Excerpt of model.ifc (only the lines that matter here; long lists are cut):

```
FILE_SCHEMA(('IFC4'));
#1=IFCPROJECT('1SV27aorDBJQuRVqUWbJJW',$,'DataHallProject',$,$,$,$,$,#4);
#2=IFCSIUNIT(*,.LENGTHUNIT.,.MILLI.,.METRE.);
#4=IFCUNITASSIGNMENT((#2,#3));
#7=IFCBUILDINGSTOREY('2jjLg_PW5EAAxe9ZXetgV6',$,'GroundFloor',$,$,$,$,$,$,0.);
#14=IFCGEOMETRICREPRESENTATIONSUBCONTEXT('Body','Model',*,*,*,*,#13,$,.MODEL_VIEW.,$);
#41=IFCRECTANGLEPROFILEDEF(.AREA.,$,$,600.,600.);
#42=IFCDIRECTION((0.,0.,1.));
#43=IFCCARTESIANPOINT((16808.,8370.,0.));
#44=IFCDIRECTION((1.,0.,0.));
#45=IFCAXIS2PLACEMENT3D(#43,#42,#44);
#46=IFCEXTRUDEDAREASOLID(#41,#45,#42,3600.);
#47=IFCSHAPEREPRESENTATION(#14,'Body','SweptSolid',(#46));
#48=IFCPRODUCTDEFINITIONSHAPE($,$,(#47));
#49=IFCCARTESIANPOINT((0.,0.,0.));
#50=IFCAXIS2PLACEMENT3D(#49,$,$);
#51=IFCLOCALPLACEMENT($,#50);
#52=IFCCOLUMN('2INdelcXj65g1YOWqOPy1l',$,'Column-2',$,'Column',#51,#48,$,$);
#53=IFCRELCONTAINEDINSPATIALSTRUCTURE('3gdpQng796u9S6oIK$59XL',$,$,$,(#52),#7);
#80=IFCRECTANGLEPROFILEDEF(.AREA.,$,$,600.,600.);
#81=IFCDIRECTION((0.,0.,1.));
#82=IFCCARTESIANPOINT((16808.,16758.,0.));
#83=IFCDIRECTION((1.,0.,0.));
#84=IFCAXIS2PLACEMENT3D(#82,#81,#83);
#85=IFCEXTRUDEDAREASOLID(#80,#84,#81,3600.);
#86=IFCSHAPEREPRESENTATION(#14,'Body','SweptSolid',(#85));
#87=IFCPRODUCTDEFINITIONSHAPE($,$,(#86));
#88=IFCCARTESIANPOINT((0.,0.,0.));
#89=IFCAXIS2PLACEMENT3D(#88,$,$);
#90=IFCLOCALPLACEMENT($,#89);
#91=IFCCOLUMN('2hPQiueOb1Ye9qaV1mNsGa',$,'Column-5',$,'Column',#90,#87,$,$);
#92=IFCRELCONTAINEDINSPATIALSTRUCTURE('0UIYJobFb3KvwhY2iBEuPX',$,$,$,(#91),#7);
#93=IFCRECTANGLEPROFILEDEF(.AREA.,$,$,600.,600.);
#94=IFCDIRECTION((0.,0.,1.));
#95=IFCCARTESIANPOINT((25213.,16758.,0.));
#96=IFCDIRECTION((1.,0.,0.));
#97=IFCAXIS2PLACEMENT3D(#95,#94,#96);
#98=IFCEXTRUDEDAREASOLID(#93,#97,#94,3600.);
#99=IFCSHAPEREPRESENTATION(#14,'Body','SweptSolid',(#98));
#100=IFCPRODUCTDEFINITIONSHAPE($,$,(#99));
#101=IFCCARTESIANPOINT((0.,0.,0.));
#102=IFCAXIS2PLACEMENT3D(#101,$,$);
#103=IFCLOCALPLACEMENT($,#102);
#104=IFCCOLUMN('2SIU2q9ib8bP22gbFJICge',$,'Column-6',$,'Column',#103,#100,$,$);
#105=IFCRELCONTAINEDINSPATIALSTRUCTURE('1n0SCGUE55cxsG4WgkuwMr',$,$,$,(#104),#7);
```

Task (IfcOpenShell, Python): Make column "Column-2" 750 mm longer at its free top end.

```python
import ifcopenshell
import ifcopenshell.util.representation
import ifcopenshell.util.unit

model = ifcopenshell.open("model.ifc")
unit_scale = ifcopenshell.util.unit.calculate_unit_scale(model)

member = model.by_id(52)
change = 0.75 / unit_scale

# The extrusion runs towards the end named, so only its depth changes.
body = ifcopenshell.util.representation.get_representation(member, "Model", "Body")
solid = body.Items[0]
old_length = solid.Depth
solid.Depth += change

print(f"length {old_length:g} -> {solid.Depth:g}")

model.write("model_updated.ifc")
```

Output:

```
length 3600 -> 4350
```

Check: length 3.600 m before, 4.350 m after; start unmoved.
